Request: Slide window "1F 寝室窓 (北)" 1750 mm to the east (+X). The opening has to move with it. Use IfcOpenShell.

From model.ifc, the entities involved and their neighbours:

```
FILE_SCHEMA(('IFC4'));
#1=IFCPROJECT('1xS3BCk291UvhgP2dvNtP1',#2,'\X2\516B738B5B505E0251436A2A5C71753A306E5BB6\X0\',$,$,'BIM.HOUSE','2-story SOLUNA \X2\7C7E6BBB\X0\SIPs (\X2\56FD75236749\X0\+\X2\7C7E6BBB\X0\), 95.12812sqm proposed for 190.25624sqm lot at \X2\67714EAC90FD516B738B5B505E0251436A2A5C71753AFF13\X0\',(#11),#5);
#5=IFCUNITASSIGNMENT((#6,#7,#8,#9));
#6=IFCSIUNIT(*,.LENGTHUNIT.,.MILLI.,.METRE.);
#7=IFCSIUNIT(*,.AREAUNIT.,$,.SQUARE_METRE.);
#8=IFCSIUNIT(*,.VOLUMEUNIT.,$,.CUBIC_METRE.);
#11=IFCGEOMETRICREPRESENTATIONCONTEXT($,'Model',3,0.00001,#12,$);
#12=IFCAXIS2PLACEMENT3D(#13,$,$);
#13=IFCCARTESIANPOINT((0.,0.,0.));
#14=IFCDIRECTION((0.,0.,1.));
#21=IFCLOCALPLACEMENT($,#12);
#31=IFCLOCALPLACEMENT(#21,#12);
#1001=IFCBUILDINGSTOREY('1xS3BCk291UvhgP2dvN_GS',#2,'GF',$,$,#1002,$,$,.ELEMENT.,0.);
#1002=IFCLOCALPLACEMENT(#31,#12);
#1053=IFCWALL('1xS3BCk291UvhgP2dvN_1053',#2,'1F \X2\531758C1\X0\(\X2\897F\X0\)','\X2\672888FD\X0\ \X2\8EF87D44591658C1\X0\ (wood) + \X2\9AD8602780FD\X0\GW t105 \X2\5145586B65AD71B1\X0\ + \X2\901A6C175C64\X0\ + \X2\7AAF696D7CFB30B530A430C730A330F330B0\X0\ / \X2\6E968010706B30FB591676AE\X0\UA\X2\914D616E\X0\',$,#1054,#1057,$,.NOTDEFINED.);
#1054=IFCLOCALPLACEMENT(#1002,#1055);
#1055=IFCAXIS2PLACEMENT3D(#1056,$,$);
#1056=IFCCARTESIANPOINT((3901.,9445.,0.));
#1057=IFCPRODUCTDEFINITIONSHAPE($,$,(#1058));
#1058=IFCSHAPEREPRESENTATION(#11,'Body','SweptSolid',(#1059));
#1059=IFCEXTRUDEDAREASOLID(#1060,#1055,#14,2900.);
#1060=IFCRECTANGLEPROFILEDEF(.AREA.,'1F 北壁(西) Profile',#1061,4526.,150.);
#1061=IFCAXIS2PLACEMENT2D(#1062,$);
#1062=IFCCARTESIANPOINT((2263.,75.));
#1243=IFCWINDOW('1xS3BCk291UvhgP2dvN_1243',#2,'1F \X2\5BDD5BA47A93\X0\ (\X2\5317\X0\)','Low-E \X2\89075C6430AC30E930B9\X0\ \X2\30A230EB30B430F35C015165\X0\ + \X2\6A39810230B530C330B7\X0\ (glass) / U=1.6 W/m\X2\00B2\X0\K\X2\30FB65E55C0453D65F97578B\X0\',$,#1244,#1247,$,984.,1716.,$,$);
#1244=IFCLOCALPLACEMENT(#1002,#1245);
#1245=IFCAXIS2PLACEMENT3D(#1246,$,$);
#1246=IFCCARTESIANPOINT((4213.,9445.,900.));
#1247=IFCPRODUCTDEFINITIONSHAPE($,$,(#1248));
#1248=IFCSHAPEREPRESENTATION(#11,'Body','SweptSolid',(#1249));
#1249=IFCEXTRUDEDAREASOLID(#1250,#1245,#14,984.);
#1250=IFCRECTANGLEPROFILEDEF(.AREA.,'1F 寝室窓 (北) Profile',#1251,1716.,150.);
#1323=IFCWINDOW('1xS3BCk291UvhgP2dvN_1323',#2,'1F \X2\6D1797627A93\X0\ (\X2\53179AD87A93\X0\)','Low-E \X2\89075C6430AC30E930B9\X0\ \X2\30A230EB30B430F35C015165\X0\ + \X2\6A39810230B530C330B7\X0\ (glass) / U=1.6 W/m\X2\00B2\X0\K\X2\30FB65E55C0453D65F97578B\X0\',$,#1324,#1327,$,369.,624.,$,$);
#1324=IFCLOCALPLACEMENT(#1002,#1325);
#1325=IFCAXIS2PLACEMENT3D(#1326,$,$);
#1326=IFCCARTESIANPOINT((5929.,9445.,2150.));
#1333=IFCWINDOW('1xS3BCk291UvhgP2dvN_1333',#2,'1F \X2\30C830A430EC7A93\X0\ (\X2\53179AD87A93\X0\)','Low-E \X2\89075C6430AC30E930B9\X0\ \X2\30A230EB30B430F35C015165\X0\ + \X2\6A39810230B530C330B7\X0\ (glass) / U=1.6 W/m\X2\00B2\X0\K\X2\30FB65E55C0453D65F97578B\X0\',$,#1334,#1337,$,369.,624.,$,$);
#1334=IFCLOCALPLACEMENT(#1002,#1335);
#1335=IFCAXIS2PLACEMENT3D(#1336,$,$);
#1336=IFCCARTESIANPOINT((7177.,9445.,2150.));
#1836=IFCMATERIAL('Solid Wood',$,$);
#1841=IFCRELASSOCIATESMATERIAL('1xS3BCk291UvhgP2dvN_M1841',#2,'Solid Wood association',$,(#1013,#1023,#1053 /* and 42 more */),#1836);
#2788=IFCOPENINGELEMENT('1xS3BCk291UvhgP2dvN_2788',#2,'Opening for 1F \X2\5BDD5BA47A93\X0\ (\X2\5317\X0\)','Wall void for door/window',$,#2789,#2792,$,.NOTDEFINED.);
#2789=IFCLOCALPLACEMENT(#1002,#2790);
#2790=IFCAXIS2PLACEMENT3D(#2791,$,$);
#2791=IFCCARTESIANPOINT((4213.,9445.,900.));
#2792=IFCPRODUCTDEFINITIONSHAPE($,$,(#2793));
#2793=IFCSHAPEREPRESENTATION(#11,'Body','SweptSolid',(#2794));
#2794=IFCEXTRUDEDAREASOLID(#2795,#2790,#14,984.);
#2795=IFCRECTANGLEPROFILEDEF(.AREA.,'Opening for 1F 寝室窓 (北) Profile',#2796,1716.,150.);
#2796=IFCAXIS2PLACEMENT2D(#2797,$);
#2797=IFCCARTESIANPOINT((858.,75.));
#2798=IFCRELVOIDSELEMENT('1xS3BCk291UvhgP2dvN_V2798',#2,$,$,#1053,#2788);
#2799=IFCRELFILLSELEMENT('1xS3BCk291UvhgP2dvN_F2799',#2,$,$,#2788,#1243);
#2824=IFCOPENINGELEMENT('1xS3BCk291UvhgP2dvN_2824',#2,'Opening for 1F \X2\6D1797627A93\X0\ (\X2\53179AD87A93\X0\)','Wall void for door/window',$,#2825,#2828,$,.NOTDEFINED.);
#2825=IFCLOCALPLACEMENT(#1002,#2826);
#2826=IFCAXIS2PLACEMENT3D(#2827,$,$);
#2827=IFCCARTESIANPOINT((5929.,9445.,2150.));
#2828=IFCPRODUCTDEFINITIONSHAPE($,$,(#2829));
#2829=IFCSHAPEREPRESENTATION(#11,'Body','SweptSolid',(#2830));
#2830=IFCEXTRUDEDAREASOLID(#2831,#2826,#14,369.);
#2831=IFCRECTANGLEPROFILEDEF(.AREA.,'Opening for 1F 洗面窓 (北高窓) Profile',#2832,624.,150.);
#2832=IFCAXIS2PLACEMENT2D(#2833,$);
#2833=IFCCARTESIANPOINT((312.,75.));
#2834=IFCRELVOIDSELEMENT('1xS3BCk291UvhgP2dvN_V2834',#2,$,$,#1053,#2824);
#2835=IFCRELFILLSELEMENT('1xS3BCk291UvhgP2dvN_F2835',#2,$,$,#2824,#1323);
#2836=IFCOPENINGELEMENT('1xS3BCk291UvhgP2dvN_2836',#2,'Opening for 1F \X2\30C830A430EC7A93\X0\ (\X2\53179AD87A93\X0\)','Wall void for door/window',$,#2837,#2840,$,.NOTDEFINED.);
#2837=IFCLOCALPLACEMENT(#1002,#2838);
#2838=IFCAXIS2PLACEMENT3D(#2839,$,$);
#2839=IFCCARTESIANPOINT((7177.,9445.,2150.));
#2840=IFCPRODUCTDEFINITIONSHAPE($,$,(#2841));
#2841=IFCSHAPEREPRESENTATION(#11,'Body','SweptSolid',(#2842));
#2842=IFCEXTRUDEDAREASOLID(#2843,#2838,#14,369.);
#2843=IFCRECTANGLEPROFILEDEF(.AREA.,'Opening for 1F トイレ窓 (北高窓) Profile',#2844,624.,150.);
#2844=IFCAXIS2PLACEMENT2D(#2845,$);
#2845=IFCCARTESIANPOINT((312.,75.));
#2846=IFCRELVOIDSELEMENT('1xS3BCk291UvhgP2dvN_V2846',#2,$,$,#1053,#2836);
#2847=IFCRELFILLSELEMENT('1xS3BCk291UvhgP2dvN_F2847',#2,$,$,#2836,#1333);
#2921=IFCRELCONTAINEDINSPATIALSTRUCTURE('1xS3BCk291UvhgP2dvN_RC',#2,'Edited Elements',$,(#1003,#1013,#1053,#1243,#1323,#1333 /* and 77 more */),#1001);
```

```python
import ifcopenshell
import ifcopenshell.api.geometry
import ifcopenshell.util.placement
import ifcopenshell.util.unit

model = ifcopenshell.open("model.ifc")
unit_scale = ifcopenshell.util.unit.calculate_unit_scale(model)

window = model.by_guid("1xS3BCk291UvhgP2dvN_1243")
opening = window.FillsVoids[0].RelatingOpeningElement
wall = opening.VoidsElements[0].RelatingBuildingElement

wall_matrix = ifcopenshell.util.placement.get_local_placement(wall.ObjectPlacement)
shift = wall_matrix[:3, 0] * 1.75 / unit_scale
before = ifcopenshell.util.placement.get_local_placement(window.ObjectPlacement)[:3, 3].copy()

# The window is not placed relative to its opening, so move both.
for product in (opening, window):
    matrix = ifcopenshell.util.placement.get_local_placement(product.ObjectPlacement)
    matrix[:3, 3] += shift
    ifcopenshell.api.geometry.edit_object_placement(model, product=product, matrix=matrix, is_si=False)

after = ifcopenshell.util.placement.get_local_placement(window.ObjectPlacement)[:3, 3]
print("window moved by", (after - before).round(3) + 0.0)

model.write("model_updated.ifc")
```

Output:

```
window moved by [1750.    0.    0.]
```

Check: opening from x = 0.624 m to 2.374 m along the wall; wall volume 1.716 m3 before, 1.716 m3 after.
